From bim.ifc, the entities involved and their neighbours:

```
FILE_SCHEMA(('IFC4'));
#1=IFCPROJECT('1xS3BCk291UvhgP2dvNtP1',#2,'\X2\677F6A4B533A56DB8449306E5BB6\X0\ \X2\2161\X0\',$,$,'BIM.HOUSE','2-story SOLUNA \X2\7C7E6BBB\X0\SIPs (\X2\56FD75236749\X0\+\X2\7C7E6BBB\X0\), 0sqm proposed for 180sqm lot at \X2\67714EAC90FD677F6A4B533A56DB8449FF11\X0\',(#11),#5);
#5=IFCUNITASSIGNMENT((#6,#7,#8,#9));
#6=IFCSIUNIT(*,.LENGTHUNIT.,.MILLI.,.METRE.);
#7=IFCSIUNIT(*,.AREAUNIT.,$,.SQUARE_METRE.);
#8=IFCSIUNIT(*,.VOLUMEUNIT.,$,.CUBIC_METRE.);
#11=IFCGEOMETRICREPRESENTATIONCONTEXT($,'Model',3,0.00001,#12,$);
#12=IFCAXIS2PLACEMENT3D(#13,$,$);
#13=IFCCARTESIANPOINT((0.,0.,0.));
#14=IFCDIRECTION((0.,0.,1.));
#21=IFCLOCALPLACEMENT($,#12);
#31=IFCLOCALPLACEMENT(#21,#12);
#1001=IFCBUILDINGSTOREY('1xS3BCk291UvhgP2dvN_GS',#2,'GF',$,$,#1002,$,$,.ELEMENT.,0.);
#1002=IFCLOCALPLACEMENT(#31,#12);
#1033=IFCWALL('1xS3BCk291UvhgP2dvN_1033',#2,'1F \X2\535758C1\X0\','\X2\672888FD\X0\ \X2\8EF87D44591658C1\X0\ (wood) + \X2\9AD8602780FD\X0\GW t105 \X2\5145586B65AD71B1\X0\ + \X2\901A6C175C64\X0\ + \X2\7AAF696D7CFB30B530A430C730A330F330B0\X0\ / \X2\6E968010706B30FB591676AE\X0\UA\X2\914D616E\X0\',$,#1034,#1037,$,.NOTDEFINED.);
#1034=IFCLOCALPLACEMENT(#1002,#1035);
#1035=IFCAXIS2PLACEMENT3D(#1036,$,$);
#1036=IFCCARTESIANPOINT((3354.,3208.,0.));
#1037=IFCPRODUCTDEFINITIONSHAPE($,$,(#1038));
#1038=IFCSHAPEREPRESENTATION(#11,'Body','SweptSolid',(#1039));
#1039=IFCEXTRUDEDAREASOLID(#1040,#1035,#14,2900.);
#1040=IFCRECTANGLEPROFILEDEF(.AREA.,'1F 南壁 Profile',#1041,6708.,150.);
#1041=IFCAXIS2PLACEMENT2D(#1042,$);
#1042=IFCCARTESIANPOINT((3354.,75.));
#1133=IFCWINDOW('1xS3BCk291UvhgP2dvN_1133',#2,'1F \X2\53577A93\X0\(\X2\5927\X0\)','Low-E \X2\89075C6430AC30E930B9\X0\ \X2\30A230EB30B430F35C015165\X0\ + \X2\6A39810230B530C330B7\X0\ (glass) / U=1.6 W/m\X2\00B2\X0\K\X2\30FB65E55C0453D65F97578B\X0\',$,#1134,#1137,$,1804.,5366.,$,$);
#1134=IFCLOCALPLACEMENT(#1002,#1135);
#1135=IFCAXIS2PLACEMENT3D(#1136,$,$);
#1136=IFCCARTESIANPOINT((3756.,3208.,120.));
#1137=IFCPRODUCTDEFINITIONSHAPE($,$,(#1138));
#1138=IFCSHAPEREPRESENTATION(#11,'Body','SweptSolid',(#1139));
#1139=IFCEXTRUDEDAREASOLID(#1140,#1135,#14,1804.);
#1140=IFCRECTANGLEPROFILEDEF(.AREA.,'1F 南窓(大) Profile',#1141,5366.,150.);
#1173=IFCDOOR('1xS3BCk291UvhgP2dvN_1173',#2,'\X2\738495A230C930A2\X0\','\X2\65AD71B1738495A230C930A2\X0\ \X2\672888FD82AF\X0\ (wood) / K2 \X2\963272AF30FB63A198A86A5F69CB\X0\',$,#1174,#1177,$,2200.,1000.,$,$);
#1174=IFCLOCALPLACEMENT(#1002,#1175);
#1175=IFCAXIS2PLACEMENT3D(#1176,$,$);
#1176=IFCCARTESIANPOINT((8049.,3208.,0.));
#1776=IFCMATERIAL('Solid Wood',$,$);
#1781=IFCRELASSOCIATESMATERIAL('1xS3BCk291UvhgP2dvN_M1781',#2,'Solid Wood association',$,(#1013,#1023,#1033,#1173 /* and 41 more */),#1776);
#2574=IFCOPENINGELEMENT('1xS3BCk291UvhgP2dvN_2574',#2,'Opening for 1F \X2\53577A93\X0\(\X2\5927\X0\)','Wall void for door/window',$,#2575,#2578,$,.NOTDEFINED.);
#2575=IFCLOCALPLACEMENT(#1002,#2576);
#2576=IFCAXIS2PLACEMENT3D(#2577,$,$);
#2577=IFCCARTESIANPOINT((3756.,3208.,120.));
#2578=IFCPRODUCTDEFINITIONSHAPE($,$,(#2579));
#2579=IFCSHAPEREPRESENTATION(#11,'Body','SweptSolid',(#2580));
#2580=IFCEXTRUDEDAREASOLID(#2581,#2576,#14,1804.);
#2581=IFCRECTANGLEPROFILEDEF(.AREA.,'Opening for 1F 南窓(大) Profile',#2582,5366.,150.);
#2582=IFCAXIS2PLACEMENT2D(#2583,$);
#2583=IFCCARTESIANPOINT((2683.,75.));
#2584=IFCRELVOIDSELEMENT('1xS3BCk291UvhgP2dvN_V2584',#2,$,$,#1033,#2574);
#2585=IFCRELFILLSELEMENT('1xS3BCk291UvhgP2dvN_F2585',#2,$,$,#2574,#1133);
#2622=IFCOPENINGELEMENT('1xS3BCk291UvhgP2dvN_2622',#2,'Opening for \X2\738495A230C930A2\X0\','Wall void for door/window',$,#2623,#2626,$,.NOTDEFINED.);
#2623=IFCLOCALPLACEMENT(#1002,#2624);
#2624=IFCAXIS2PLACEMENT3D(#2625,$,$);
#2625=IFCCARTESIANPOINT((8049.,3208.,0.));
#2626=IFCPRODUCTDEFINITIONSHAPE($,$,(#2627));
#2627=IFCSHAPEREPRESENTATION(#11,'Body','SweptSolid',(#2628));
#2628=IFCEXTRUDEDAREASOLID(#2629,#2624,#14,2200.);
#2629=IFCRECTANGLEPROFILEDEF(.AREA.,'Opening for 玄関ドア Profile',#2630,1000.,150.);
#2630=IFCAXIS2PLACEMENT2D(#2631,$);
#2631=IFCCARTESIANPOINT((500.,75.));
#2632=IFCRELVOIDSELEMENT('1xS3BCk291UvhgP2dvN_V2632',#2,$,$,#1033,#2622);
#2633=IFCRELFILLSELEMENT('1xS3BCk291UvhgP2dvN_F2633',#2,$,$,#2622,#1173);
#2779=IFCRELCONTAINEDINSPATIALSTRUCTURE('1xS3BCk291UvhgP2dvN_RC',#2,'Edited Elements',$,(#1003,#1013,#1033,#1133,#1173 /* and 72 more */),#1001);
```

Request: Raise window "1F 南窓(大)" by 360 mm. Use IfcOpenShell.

```python
import numpy as np
import ifcopenshell
import ifcopenshell.api.geometry
import ifcopenshell.util.placement
import ifcopenshell.util.unit

model = ifcopenshell.open("bim.ifc")
unit_scale = ifcopenshell.util.unit.calculate_unit_scale(model)

window = model.by_guid("1xS3BCk291UvhgP2dvN_1133")
opening = window.FillsVoids[0].RelatingOpeningElement
dz = 0.36 / unit_scale

shift = np.array([0.0, 0.0, dz])
# The window is not placed relative to its opening, so move both.
for product in (opening, window):
    matrix = ifcopenshell.util.placement.get_local_placement(product.ObjectPlacement)
    matrix[:3, 3] += shift
    ifcopenshell.api.geometry.edit_object_placement(model, product=product, matrix=matrix, is_si=False)

print(f"moved by {dz * unit_scale:+.3f} m")

model.write("bim-out.ifc")
```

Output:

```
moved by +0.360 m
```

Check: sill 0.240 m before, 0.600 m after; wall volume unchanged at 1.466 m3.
